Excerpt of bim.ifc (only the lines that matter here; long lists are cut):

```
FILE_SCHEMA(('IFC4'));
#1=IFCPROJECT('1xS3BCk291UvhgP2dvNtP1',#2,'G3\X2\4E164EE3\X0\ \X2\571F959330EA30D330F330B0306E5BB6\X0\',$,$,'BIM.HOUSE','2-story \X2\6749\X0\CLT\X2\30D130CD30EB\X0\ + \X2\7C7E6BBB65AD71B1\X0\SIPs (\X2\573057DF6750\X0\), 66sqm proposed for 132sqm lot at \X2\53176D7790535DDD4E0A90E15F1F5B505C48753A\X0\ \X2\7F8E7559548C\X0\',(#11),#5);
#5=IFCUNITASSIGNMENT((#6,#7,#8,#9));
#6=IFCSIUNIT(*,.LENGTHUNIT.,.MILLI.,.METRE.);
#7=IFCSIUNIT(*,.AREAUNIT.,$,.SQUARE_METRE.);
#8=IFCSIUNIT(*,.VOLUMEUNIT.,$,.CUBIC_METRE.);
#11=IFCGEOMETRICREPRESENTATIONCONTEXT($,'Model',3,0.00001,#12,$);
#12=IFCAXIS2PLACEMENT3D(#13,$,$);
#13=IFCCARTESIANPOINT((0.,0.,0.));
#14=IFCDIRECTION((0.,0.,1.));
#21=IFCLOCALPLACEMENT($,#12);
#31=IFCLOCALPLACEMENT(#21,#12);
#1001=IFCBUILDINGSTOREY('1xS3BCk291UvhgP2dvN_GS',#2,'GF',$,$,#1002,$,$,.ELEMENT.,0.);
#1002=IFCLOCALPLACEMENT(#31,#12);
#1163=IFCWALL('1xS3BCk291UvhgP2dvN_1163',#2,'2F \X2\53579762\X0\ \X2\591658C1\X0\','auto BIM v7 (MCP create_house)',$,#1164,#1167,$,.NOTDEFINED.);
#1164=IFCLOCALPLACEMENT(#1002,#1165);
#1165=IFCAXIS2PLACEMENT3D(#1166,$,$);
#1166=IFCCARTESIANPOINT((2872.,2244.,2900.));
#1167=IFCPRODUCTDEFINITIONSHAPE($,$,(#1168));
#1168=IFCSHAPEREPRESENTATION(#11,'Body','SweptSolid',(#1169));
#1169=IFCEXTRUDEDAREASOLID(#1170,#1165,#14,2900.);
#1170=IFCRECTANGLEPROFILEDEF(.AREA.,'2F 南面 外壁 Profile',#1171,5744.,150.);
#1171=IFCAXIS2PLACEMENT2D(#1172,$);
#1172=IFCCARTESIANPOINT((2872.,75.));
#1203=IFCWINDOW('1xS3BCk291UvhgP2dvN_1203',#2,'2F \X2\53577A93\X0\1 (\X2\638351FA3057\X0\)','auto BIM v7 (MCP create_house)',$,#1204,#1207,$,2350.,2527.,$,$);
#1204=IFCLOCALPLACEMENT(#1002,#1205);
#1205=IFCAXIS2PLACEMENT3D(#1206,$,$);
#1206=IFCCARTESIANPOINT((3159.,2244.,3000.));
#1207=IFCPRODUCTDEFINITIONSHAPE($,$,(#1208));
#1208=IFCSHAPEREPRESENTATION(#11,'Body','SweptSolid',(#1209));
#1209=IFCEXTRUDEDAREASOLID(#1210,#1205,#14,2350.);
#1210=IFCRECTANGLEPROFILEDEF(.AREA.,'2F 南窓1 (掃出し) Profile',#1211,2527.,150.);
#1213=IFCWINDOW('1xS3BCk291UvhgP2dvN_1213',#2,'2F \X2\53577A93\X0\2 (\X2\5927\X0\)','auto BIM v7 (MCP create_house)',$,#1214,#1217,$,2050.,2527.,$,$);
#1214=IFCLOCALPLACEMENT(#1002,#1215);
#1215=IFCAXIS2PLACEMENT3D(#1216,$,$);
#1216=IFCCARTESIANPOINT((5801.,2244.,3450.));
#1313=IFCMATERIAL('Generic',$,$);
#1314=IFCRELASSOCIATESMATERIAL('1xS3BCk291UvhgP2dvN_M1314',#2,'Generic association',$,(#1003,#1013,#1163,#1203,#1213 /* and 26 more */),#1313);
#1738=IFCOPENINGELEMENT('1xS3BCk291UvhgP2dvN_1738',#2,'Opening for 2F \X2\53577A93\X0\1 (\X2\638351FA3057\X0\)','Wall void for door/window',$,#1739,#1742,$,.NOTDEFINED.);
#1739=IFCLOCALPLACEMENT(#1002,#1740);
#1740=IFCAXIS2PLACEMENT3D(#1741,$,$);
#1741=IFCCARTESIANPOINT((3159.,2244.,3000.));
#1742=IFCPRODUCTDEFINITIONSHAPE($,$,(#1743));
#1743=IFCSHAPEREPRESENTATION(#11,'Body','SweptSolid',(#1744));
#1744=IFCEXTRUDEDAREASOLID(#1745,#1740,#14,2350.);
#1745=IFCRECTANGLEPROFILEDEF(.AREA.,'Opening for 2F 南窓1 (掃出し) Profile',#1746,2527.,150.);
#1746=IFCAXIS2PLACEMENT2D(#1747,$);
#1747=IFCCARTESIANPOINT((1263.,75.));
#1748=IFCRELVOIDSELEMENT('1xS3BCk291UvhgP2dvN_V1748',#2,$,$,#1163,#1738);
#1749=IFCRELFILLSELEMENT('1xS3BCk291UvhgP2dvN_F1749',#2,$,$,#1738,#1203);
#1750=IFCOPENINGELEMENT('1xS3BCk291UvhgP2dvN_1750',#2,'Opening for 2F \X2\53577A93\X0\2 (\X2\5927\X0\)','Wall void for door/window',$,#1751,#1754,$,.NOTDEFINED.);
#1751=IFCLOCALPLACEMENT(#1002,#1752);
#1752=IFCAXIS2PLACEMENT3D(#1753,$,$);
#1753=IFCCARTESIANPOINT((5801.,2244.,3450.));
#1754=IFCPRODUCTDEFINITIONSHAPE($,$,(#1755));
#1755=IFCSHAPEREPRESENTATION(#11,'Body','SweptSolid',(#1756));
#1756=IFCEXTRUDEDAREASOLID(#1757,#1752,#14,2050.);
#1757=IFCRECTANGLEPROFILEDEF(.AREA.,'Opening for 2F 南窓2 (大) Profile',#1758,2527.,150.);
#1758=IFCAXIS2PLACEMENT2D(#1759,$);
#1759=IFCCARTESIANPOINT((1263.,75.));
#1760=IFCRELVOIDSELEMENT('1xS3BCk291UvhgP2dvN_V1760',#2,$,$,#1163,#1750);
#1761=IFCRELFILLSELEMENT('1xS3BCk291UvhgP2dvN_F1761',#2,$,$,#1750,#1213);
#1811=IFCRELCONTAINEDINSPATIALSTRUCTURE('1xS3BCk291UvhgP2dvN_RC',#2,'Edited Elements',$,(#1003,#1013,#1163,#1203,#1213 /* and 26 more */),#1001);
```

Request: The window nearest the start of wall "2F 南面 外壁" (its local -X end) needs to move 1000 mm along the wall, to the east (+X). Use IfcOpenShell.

```python
import ifcopenshell
import ifcopenshell.api.geometry
import ifcopenshell.util.placement
import ifcopenshell.util.unit

model = ifcopenshell.open("bim.ifc")
unit_scale = ifcopenshell.util.unit.calculate_unit_scale(model)

window = model.by_guid("1xS3BCk291UvhgP2dvN_1203")
opening = window.FillsVoids[0].RelatingOpeningElement
wall = opening.VoidsElements[0].RelatingBuildingElement

wall_matrix = ifcopenshell.util.placement.get_local_placement(wall.ObjectPlacement)
shift = wall_matrix[:3, 0] * 1 / unit_scale
before = ifcopenshell.util.placement.get_local_placement(window.ObjectPlacement)[:3, 3].copy()

# The window is not placed relative to its opening, so move both.
for product in (opening, window):
    matrix = ifcopenshell.util.placement.get_local_placement(product.ObjectPlacement)
    matrix[:3, 3] += shift
    ifcopenshell.api.geometry.edit_object_placement(model, product=product, matrix=matrix, is_si=False)

after = ifcopenshell.util.placement.get_local_placement(window.ObjectPlacement)[:3, 3]
print("window moved by", (after - before).round(3) + 0.0)

model.write("bim_edited.ifc")
```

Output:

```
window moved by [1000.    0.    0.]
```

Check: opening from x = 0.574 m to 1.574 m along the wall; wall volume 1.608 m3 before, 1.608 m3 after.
